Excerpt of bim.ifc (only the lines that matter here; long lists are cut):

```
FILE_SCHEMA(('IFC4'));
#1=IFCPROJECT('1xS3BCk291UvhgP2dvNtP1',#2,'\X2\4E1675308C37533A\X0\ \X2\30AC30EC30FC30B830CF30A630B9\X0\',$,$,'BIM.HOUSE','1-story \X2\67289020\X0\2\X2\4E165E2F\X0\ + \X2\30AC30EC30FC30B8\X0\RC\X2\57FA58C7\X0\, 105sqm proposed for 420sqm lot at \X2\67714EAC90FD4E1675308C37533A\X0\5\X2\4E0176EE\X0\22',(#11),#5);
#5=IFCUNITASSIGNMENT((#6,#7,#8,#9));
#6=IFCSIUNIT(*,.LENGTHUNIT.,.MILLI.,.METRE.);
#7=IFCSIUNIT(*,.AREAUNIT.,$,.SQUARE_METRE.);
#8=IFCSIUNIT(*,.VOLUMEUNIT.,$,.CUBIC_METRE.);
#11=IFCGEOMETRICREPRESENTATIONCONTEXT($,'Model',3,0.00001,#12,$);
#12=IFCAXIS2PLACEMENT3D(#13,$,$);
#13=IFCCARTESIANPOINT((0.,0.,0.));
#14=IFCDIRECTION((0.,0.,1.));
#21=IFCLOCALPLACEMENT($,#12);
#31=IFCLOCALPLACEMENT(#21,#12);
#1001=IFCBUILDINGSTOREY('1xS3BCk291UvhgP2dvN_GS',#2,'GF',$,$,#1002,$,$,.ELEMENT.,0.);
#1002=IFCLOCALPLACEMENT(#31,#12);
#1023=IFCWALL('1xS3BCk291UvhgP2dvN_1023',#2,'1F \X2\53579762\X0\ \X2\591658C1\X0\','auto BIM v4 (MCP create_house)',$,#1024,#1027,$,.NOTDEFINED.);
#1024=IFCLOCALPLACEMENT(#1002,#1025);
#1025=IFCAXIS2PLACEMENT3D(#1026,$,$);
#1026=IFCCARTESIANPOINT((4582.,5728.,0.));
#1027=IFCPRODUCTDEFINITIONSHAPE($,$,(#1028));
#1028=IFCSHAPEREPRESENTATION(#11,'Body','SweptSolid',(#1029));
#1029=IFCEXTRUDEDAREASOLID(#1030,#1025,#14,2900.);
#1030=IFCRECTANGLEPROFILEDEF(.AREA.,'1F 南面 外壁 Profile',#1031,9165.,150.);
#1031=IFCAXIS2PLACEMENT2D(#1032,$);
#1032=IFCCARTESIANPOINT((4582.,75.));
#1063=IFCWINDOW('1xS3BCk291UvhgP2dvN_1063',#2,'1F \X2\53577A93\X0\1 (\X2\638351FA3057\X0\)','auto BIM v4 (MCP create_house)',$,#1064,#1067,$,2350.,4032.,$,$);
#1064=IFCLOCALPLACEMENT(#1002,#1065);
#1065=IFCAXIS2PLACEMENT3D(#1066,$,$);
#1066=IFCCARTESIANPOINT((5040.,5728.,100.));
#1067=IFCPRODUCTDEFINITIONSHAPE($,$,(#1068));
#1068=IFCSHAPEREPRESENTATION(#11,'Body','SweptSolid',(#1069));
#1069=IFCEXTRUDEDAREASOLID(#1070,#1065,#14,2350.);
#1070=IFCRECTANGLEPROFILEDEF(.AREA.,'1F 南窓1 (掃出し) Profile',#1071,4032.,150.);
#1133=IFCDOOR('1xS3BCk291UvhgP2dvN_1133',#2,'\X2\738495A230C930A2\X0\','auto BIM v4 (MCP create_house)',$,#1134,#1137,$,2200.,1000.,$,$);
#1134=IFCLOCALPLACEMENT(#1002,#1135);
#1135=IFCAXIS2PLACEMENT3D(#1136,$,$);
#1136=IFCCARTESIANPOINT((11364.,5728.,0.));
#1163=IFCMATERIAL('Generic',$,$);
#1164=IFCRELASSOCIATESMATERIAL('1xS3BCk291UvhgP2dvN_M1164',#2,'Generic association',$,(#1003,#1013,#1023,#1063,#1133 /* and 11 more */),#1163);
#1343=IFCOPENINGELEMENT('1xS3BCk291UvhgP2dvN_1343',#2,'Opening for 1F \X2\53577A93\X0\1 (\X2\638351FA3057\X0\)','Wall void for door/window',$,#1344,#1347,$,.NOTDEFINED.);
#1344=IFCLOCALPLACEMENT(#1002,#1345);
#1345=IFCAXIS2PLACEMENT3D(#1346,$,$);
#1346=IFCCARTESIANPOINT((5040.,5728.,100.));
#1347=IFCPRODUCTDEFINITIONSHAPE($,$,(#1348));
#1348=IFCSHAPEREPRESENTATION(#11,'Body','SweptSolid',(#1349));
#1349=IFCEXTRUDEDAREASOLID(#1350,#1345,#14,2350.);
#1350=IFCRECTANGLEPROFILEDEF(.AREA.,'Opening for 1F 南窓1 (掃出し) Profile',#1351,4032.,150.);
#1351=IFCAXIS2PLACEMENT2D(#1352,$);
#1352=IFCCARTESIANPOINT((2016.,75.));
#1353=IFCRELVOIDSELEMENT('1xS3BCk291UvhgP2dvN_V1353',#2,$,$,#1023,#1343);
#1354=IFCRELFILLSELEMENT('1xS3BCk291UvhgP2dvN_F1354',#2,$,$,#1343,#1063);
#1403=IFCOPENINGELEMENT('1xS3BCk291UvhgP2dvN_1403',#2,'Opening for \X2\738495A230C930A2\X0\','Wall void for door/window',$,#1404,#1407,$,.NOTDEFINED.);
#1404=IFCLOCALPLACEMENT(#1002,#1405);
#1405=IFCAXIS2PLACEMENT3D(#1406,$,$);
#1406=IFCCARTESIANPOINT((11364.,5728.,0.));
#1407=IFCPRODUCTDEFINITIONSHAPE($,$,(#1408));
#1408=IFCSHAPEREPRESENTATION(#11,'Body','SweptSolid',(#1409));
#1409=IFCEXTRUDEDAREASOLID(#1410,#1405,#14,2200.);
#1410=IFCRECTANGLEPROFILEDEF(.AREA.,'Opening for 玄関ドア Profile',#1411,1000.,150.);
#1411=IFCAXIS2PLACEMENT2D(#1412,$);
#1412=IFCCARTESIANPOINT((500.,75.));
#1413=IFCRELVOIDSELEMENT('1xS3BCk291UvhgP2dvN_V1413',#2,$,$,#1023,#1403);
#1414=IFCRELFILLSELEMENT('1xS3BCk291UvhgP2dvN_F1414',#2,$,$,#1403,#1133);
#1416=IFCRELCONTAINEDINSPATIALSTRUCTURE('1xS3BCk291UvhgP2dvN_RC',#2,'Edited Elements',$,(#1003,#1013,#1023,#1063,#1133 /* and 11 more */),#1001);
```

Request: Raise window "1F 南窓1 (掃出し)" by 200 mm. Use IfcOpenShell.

```python
import numpy as np
import ifcopenshell
import ifcopenshell.api.geometry
import ifcopenshell.util.placement
import ifcopenshell.util.unit

model = ifcopenshell.open("bim.ifc")
unit_scale = ifcopenshell.util.unit.calculate_unit_scale(model)

window = model.by_guid("1xS3BCk291UvhgP2dvN_1063")
opening = window.FillsVoids[0].RelatingOpeningElement
dz = 0.2 / unit_scale

shift = np.array([0.0, 0.0, dz])
# The window is not placed relative to its opening, so move both.
for product in (opening, window):
    matrix = ifcopenshell.util.placement.get_local_placement(product.ObjectPlacement)
    matrix[:3, 3] += shift
    ifcopenshell.api.geometry.edit_object_placement(model, product=product, matrix=matrix, is_si=False)

print(f"moved by {dz * unit_scale:+.3f} m")

model.write("bim_v2.ifc")
```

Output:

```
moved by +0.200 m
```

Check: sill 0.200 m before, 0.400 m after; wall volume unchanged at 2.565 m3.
